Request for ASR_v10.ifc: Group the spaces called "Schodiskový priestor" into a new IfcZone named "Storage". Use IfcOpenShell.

First a look at what the model holds.

```python
import ifcopenshell

model = ifcopenshell.open("ASR_v10.ifc")
print(model.schema)
seen = {}
for space in model.by_type("IfcSpace"):
    seen[space.LongName] = seen.get(space.LongName, 0) + 1
for name, count in sorted(seen.items(), key=str):
    print(count, "x", name)
print("zones:", [z.Name for z in model.by_type("IfcZone")][:20])
```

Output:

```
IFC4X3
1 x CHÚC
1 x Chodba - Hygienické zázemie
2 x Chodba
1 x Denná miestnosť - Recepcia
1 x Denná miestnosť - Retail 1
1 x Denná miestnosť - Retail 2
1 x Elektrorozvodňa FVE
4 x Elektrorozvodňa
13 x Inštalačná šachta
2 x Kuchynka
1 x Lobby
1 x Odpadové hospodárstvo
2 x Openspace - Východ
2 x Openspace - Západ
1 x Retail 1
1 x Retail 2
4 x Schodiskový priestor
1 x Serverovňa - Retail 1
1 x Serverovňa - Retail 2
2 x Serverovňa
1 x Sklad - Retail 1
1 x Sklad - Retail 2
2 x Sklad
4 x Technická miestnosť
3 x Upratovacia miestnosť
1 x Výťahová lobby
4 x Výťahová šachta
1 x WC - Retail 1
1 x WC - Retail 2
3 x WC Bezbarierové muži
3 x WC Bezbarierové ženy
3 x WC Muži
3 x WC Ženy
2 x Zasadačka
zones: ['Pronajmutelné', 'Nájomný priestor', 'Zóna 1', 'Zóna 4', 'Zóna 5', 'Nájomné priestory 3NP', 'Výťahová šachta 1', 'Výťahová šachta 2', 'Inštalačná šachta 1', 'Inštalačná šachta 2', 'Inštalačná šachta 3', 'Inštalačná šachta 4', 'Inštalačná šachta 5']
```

```python
import ifcopenshell
import ifcopenshell.api.group
import ifcopenshell.api.root

model = ifcopenshell.open("ASR_v10.ifc")

names = {"Schodiskový priestor"}
spaces = [s for s in model.by_type("IfcSpace") if s.LongName in names]

zone = ifcopenshell.api.root.create_entity(model, ifc_class="IfcZone", name="Storage")
ifcopenshell.api.group.assign_group(model, products=spaces, group=zone)
print(len(spaces), "spaces in", zone.Name)

model.write("ASR_v10_edited.ifc")
```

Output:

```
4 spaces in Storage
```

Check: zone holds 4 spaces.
